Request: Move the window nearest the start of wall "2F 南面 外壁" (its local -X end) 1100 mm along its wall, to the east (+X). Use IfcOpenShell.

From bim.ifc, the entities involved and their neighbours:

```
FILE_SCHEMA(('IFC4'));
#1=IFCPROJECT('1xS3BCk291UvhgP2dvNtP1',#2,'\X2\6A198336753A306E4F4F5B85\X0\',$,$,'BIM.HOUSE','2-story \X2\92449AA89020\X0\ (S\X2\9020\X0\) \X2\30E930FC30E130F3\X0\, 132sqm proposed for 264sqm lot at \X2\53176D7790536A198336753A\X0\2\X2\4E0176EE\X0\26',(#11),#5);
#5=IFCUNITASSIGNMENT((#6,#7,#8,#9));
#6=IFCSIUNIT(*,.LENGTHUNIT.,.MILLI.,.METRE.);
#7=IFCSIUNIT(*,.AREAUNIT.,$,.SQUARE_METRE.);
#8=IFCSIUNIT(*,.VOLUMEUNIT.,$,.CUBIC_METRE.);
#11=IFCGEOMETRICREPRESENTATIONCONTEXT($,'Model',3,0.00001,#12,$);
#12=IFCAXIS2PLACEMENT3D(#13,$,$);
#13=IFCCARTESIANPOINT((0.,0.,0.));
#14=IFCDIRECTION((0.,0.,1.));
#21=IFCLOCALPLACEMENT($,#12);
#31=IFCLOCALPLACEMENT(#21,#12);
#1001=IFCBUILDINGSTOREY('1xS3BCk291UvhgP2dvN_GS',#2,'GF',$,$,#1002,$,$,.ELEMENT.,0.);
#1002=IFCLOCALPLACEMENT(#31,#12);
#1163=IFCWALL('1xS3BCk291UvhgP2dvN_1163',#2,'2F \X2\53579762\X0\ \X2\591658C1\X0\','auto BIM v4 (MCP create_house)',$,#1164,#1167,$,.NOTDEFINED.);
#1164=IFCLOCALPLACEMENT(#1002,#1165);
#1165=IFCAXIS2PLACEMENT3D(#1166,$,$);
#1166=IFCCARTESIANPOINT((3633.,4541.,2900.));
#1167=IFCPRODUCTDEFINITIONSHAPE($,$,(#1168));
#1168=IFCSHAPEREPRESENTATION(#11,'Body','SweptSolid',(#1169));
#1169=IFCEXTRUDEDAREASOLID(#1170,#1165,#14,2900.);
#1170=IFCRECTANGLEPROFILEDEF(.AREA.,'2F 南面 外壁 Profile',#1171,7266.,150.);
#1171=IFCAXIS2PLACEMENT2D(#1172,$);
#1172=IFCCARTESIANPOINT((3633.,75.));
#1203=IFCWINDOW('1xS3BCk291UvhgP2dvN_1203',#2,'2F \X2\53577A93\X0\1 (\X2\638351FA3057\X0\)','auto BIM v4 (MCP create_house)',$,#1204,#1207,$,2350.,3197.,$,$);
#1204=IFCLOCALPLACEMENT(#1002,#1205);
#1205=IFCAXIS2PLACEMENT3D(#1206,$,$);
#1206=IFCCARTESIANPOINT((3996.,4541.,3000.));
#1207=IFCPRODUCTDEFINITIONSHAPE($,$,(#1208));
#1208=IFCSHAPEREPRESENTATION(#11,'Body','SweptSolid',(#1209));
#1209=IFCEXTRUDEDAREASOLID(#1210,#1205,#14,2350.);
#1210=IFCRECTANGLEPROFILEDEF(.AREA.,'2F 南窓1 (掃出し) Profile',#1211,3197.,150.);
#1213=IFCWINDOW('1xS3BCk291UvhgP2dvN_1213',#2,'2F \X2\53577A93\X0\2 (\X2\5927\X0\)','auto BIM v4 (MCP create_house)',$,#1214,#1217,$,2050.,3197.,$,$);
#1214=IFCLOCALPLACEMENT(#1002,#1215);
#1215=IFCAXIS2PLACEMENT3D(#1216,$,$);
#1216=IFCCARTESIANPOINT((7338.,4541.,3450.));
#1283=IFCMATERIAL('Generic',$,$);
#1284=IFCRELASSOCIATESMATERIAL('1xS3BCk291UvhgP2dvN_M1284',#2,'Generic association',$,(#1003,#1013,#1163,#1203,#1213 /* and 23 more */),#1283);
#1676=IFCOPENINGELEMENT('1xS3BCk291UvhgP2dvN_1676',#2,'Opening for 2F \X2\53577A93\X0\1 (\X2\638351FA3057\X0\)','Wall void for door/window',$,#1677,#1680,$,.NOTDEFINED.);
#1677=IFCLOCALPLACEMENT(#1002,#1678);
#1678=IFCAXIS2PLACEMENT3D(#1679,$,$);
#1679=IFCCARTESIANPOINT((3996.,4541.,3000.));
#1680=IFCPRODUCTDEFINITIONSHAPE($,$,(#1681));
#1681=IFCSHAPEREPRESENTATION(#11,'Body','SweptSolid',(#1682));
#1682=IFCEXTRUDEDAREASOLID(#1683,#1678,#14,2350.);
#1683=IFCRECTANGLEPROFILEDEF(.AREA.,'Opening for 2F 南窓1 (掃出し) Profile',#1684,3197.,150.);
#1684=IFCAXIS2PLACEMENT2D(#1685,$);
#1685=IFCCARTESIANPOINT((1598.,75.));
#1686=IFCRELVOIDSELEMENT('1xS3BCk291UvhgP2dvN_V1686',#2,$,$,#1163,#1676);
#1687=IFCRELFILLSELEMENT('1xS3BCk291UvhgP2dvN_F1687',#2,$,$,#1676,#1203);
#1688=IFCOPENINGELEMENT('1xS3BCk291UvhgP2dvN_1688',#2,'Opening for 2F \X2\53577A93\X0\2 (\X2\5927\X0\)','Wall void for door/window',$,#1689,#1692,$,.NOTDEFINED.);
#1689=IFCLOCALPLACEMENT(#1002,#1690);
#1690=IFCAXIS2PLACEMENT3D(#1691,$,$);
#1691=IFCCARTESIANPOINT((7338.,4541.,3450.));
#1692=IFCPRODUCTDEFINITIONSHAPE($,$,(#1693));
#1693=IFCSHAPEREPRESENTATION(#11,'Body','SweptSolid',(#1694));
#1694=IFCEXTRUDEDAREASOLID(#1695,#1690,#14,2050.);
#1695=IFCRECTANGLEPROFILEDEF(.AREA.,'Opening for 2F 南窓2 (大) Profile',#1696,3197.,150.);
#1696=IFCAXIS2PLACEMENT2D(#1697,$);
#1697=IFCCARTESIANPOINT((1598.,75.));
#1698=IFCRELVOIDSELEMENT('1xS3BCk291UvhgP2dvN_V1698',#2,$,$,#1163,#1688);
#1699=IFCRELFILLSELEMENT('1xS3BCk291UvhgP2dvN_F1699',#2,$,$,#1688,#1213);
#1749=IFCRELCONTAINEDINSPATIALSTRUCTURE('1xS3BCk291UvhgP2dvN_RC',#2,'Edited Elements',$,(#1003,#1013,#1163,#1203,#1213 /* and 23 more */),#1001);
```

```python
import ifcopenshell
import ifcopenshell.api.geometry
import ifcopenshell.util.placement
import ifcopenshell.util.unit

model = ifcopenshell.open("bim.ifc")
unit_scale = ifcopenshell.util.unit.calculate_unit_scale(model)

window = model.by_guid("1xS3BCk291UvhgP2dvN_1203")
opening = window.FillsVoids[0].RelatingOpeningElement
wall = opening.VoidsElements[0].RelatingBuildingElement

wall_matrix = ifcopenshell.util.placement.get_local_placement(wall.ObjectPlacement)
shift = wall_matrix[:3, 0] * 1.1 / unit_scale
before = ifcopenshell.util.placement.get_local_placement(window.ObjectPlacement)[:3, 3].copy()

# The window is not placed relative to its opening, so move both.
for product in (opening, window):
    matrix = ifcopenshell.util.placement.get_local_placement(product.ObjectPlacement)
    matrix[:3, 3] += shift
    ifcopenshell.api.geometry.edit_object_placement(model, product=product, matrix=matrix, is_si=False)

after = ifcopenshell.util.placement.get_local_placement(window.ObjectPlacement)[:3, 3]
print("window moved by", (after - before).round(3) + 0.0)

model.write("bim-out.ifc")
```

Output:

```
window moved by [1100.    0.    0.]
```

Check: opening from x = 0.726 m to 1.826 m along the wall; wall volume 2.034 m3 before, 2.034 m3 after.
